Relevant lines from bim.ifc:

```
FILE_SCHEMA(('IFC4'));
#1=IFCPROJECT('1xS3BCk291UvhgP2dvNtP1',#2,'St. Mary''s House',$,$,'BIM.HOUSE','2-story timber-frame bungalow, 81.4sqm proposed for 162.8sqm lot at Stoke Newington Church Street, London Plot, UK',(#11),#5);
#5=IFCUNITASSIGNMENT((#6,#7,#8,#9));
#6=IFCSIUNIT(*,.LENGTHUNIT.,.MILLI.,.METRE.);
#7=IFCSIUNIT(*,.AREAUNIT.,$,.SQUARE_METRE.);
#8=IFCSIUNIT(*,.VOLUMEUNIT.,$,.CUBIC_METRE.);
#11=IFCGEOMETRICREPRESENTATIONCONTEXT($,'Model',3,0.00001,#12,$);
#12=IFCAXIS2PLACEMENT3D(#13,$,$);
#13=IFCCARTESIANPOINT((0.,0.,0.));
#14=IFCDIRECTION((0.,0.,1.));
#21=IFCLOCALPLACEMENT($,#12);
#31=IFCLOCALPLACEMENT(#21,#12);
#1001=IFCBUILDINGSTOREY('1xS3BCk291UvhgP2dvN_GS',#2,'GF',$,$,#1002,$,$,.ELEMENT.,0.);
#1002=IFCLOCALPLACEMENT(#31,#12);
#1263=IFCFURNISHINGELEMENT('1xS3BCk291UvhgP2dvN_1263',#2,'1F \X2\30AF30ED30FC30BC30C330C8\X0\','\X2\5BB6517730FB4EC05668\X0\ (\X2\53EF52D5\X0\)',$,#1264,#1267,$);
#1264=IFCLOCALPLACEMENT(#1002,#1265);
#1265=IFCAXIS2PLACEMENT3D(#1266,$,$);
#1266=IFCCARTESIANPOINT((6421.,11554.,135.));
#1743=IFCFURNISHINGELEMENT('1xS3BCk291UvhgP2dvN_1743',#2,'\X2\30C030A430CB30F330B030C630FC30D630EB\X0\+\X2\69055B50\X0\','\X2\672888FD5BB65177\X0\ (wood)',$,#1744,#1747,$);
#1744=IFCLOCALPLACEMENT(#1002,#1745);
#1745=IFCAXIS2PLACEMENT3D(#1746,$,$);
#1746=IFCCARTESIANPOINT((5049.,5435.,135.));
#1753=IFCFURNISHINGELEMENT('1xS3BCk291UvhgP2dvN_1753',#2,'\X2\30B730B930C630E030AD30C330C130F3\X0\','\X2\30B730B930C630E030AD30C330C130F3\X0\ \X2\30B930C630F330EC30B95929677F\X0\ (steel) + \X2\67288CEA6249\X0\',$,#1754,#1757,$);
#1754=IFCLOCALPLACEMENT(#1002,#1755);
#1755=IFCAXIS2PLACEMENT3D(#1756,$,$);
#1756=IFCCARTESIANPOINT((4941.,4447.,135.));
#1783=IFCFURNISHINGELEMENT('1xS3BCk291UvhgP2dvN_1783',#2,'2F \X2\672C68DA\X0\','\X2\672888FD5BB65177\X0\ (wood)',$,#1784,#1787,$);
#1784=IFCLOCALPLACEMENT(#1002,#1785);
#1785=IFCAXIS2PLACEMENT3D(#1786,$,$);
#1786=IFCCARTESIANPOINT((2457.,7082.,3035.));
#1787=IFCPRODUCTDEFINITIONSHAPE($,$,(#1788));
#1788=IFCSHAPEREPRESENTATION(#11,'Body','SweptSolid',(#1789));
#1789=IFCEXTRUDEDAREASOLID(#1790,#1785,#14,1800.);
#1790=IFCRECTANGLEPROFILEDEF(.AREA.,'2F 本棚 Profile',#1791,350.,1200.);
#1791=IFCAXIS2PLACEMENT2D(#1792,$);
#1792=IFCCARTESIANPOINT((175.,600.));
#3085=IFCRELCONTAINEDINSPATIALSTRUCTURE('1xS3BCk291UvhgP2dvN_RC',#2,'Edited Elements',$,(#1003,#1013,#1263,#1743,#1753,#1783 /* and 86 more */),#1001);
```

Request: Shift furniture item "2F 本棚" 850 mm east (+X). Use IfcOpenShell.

```python
import ifcopenshell
import ifcopenshell.api.geometry
import ifcopenshell.util.placement
import ifcopenshell.util.unit

model = ifcopenshell.open("bim.ifc")
unit_scale = ifcopenshell.util.unit.calculate_unit_scale(model)

item = model.by_guid("1xS3BCk291UvhgP2dvN_1783")
matrix = ifcopenshell.util.placement.get_local_placement(item.ObjectPlacement)
matrix[0, 3] += 0.85 / unit_scale
ifcopenshell.api.geometry.edit_object_placement(model, product=item, matrix=matrix, is_si=False)

print(ifcopenshell.util.placement.get_local_placement(item.ObjectPlacement).round(3) + 0.0)

model.write("bim-out.ifc")
```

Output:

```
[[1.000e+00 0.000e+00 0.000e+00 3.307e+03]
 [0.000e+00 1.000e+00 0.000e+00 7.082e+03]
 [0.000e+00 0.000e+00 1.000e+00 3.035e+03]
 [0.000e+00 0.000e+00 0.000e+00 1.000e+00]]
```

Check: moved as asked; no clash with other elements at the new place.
